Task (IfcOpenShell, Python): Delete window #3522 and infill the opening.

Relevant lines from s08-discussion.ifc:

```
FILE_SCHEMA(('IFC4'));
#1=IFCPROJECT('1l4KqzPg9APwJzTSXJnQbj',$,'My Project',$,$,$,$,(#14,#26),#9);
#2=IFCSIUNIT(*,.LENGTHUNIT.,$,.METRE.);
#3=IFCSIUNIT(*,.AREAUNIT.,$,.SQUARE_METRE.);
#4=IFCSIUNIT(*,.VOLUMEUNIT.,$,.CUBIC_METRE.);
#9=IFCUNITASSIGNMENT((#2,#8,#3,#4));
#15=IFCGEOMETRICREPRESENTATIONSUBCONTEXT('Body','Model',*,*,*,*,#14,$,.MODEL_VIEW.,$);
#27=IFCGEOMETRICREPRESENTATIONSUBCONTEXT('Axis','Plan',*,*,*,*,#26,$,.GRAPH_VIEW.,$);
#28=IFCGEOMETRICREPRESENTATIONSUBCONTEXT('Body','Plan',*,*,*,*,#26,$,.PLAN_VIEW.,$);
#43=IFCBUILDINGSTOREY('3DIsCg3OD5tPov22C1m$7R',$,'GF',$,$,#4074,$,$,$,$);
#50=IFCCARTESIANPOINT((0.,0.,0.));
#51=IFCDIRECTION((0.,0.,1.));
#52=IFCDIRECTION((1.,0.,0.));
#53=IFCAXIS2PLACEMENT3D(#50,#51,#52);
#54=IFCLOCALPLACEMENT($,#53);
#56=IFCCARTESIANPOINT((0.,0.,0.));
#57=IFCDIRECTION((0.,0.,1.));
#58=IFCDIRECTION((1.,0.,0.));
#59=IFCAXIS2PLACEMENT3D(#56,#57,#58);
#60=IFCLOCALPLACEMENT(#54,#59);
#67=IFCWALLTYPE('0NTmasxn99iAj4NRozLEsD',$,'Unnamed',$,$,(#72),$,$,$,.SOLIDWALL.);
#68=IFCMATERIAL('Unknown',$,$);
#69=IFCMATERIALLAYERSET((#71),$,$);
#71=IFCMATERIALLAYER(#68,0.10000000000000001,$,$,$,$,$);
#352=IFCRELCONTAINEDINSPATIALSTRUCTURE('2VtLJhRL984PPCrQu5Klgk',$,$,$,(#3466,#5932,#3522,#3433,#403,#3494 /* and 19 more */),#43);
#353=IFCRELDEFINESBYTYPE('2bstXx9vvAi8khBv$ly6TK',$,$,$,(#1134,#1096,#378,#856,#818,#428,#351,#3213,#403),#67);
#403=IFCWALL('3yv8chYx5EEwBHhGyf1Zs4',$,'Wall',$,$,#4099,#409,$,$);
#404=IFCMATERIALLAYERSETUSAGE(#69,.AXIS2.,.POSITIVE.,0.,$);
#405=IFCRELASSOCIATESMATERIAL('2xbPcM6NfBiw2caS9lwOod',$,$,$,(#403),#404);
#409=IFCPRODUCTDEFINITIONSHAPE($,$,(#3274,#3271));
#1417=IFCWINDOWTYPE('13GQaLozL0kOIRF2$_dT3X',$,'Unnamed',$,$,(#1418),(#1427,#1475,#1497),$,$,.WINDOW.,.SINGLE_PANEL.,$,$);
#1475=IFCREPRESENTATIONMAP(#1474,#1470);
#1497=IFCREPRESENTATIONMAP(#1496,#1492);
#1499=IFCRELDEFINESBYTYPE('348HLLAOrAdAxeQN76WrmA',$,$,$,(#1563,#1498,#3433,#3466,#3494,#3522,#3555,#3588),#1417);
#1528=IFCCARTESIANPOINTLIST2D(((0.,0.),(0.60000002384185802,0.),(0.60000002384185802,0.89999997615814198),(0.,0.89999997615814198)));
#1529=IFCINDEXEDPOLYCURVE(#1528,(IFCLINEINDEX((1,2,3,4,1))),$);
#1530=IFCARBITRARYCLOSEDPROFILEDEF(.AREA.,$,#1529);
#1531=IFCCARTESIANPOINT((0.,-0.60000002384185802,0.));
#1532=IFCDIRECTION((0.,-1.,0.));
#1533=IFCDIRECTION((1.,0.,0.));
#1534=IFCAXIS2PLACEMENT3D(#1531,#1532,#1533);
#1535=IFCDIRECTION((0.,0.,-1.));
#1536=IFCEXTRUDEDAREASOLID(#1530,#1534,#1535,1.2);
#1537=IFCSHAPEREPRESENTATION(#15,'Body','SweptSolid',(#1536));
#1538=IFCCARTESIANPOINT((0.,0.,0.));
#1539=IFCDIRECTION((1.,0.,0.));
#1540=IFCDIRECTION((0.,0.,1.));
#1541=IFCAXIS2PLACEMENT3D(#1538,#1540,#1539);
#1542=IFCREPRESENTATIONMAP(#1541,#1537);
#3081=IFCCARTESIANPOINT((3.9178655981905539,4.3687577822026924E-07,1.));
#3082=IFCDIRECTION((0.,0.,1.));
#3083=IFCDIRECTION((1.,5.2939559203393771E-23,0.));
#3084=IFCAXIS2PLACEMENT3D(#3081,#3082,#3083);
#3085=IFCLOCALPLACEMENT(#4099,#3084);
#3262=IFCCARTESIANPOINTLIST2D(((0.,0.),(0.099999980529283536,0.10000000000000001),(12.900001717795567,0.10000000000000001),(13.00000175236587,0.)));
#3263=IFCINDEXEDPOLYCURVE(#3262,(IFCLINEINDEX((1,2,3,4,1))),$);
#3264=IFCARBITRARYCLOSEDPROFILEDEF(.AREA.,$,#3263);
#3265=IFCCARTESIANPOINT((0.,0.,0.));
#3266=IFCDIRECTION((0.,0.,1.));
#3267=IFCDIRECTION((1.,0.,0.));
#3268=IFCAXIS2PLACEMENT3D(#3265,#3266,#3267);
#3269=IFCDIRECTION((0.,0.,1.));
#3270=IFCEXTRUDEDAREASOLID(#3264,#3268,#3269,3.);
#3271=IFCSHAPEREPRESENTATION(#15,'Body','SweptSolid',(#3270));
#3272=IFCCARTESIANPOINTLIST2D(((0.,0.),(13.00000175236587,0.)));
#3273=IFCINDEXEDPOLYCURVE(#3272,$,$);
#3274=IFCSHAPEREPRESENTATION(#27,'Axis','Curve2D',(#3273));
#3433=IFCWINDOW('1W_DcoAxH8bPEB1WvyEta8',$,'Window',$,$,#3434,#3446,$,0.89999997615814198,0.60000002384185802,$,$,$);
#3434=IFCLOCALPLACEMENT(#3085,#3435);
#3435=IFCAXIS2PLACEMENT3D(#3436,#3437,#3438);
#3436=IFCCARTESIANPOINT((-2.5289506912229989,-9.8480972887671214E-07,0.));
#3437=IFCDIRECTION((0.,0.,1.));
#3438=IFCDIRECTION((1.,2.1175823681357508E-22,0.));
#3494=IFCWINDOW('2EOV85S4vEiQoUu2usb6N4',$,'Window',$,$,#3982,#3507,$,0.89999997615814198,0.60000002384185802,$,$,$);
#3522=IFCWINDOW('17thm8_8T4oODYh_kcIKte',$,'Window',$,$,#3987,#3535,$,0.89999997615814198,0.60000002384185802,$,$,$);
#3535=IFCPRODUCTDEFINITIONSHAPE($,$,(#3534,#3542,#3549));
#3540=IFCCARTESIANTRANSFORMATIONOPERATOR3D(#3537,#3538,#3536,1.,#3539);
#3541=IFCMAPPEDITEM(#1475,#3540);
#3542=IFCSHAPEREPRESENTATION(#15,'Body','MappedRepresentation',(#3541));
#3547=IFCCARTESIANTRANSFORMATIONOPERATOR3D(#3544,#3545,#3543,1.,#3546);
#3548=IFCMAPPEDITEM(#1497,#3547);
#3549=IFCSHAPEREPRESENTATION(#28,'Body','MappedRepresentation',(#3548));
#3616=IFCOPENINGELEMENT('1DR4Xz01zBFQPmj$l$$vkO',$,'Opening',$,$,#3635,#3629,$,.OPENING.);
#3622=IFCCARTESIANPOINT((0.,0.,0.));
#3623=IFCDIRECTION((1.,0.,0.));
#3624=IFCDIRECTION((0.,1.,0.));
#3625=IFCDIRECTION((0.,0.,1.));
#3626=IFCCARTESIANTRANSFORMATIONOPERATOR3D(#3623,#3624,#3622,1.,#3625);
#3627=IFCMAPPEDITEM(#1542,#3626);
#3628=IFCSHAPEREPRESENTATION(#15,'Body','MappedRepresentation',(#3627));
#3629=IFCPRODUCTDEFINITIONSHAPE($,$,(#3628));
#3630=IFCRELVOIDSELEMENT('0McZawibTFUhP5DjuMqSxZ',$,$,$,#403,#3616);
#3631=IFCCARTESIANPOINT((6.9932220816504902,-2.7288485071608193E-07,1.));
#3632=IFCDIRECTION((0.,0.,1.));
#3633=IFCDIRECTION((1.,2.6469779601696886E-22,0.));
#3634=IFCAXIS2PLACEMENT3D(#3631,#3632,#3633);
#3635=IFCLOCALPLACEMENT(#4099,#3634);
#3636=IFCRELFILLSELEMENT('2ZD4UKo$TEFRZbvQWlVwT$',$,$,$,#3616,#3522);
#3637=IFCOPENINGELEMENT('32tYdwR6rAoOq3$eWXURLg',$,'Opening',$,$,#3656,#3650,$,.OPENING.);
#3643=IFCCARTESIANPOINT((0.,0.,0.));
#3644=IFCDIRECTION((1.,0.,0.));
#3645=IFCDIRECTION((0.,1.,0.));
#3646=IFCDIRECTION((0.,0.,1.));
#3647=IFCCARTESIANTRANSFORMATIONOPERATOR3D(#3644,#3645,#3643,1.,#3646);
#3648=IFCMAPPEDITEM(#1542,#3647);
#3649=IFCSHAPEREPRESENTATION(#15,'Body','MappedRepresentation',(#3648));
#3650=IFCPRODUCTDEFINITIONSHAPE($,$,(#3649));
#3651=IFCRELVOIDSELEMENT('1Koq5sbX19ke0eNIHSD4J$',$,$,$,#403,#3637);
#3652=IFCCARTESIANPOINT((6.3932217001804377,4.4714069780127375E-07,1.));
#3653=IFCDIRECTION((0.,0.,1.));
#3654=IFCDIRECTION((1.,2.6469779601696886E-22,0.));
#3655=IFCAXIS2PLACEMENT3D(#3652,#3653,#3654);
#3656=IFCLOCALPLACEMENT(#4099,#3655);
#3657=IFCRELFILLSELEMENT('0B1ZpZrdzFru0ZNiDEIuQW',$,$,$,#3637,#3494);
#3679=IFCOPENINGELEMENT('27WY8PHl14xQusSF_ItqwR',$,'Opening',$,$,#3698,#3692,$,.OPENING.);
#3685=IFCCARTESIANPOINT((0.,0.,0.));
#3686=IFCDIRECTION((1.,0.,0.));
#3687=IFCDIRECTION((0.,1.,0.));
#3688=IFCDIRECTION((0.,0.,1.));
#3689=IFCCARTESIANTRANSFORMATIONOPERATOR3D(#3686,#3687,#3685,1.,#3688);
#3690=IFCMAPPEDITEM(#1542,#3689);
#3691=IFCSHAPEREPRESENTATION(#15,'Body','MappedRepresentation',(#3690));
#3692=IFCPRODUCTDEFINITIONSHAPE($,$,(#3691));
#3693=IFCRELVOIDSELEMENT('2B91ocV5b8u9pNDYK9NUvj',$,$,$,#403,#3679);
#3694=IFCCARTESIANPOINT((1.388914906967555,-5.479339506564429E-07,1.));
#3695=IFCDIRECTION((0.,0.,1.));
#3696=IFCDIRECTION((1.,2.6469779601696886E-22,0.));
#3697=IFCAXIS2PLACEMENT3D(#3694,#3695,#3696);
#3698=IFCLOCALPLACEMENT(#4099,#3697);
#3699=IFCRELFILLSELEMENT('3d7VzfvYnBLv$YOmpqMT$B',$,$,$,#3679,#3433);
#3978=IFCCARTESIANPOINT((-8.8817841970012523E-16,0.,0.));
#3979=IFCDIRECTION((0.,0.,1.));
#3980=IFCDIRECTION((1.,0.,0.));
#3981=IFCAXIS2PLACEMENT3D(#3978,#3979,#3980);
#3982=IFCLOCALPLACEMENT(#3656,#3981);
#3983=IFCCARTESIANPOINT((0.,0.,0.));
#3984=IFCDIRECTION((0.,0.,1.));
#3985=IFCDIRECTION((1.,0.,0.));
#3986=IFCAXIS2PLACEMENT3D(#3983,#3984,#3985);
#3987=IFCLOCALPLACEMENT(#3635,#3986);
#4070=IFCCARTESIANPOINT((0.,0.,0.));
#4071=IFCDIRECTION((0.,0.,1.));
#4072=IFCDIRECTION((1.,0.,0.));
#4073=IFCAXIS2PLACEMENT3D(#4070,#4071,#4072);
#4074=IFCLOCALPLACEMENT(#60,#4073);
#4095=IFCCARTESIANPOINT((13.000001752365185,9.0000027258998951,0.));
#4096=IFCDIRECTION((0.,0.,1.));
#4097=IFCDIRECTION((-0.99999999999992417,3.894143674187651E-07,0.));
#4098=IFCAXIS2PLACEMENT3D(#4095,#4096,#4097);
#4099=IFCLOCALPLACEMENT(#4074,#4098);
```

```python
import ifcopenshell
import ifcopenshell.api.feature
import ifcopenshell.api.root
import ifcopenshell.geom
import ifcopenshell.util.shape

model = ifcopenshell.open("s08-discussion.ifc")
settings = ifcopenshell.geom.settings()


def volume(element):
    """Net volume in cubic metres, openings subtracted."""
    shape = ifcopenshell.geom.create_shape(settings, element)
    return ifcopenshell.util.shape.get_volume(shape.geometry)


window = model.by_id(3522)
opening = window.FillsVoids[0].RelatingOpeningElement
wall = opening.VoidsElements[0].RelatingBuildingElement
before = volume(wall)

ifcopenshell.api.root.remove_product(model, product=window)
ifcopenshell.api.feature.remove_feature(model, feature=opening)

after = volume(wall)

print(f"wall volume {before:.3f} -> {after:.3f} m3")

model.write("s08-discussion_updated.ifc")
```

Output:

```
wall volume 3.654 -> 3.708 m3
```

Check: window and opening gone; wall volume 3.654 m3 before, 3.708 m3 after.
